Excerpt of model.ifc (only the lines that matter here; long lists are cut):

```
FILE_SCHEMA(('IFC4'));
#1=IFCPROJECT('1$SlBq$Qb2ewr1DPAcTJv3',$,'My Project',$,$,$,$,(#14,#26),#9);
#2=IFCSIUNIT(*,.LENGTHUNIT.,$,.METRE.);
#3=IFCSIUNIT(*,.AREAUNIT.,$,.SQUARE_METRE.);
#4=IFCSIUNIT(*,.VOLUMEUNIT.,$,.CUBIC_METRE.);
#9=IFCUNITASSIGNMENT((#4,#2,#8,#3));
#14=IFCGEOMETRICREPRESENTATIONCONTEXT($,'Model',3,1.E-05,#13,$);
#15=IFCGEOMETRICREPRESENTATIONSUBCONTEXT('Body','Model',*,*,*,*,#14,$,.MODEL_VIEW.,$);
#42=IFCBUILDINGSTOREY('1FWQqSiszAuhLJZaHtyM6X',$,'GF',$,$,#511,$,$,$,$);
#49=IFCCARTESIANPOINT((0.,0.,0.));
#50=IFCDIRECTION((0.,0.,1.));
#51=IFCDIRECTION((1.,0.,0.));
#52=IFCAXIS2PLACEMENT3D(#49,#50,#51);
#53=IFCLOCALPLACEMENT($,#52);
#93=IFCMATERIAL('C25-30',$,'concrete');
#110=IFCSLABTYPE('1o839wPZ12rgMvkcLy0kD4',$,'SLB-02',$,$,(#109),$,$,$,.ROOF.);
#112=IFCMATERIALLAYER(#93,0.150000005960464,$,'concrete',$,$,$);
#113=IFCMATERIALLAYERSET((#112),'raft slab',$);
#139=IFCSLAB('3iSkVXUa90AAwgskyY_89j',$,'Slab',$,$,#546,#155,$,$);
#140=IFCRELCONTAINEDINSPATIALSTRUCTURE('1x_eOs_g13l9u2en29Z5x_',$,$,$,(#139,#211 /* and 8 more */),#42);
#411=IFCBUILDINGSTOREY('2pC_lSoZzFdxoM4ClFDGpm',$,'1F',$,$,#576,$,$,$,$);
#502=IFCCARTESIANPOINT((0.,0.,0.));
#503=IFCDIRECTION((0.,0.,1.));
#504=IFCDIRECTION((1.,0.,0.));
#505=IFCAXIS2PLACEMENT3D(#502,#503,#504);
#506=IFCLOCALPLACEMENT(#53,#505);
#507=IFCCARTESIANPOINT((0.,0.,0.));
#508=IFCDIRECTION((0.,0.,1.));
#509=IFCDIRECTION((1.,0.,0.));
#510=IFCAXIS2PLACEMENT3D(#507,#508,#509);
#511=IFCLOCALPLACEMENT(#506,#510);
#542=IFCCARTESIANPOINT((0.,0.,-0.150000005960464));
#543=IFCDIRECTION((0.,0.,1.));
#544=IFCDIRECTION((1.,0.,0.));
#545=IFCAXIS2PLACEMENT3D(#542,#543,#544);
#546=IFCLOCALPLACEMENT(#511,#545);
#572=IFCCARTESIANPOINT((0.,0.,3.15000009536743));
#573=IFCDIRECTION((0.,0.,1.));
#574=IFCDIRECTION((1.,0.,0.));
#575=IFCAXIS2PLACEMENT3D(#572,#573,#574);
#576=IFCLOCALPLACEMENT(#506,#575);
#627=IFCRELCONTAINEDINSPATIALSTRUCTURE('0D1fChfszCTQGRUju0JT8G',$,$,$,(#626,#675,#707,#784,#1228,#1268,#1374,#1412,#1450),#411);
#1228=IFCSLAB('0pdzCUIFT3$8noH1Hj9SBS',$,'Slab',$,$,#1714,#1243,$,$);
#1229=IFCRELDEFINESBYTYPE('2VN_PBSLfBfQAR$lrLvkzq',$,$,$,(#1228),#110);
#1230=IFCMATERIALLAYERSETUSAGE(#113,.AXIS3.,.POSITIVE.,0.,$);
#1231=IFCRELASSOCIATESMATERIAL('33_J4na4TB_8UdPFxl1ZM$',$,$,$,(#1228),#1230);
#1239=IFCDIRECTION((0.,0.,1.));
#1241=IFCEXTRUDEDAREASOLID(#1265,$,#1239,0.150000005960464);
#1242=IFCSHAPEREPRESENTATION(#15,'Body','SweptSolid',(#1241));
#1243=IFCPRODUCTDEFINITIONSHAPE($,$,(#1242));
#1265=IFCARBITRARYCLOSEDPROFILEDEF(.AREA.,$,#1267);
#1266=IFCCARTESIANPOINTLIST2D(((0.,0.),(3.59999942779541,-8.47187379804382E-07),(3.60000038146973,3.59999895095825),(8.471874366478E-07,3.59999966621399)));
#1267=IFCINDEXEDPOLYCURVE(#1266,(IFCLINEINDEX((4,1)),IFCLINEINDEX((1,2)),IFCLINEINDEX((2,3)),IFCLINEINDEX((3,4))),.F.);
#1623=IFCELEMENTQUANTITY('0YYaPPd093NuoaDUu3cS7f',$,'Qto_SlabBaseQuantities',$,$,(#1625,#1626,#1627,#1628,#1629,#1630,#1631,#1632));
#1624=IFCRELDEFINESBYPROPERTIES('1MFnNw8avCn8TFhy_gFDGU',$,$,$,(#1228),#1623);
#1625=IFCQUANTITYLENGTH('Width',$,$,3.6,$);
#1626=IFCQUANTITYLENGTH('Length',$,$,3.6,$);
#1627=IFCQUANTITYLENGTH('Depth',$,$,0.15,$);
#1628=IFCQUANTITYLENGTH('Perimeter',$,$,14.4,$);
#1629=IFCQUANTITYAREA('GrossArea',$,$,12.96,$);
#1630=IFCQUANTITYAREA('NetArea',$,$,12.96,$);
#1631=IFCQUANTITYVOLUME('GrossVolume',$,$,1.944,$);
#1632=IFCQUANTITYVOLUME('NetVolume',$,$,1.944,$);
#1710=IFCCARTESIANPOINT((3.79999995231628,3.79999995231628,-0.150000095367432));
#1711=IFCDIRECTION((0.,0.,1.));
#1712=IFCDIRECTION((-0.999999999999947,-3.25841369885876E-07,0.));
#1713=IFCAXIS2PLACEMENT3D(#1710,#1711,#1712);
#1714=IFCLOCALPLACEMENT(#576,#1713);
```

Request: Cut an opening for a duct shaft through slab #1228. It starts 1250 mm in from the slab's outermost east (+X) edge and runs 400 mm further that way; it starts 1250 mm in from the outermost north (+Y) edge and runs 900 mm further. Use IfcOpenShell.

```python
import numpy as np
import ifcopenshell
import ifcopenshell.api.feature
import ifcopenshell.api.geometry
import ifcopenshell.api.pset
import ifcopenshell.api.root
import ifcopenshell.geom
import ifcopenshell.util.element
import ifcopenshell.util.placement
import ifcopenshell.util.representation
import ifcopenshell.util.shape
import ifcopenshell.util.unit

model = ifcopenshell.open("model.ifc")
unit_scale = ifcopenshell.util.unit.calculate_unit_scale(model)
area_scale = ifcopenshell.util.unit.calculate_unit_scale(model, "AREAUNIT")
volume_scale = ifcopenshell.util.unit.calculate_unit_scale(model, "VOLUMEUNIT")
settings = ifcopenshell.geom.settings()


def volume(element):
    """Net volume in cubic metres, openings subtracted."""
    shape = ifcopenshell.geom.create_shape(settings, element)
    return ifcopenshell.util.shape.get_volume(shape.geometry)


slab = model.by_guid("0pdzCUIFT3$8noH1Hj9SBS")
before = volume(slab)

# Extent in the slab's own axes, in metres. The edges named are its -X and -Y sides.
slab_shape = ifcopenshell.geom.create_shape(settings, slab)
vertices = ifcopenshell.util.shape.get_vertices(slab_shape.geometry)
x_min, y_min, bottom = vertices.min(axis=0)
top = vertices[:, 2].max()

opening = ifcopenshell.api.root.create_entity(model, ifc_class="IfcOpeningElement", name="Duct shaft opening", predefined_type="OPENING")
context = ifcopenshell.util.representation.get_context(model, "Model", "Body", "MODEL_VIEW")
width, depth = 0.4, 0.9
outline = [(0.0, 0.0), (width, 0.0), (width, depth), (0.0, depth), (0.0, 0.0)]
# Overshoot both faces by 50 mm so the cut is clean.
shape = ifcopenshell.api.geometry.add_slab_representation(
    model, context=context, depth=top - bottom + 0.1, polyline=outline
)
ifcopenshell.api.geometry.assign_representation(model, product=opening, representation=shape)

matrix = ifcopenshell.util.placement.get_local_placement(slab.ObjectPlacement)
matrix[:, 3] = matrix @ np.append(np.array([x_min + 1.25, y_min + 1.25, bottom - 0.05]) / unit_scale, 1.0)
ifcopenshell.api.geometry.edit_object_placement(model, product=opening, matrix=matrix, is_si=False)
ifcopenshell.api.feature.add_feature(model, feature=opening, element=slab)

after = volume(slab)

# Update the slab's stored quantities.
qto = model.by_id(ifcopenshell.util.element.get_pset(slab, "Qto_SlabBaseQuantities", should_inherit=False)["id"])
ifcopenshell.api.pset.edit_qto(model, qto=qto, properties={
    "NetArea": after / (top - bottom) / area_scale,
    "NetVolume": after / volume_scale,
})

print(f"slab volume {before:.3f} -> {after:.3f} m3")

model.write("model_updated.ifc")
```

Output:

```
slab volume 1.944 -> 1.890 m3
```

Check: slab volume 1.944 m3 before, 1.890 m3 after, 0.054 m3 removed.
